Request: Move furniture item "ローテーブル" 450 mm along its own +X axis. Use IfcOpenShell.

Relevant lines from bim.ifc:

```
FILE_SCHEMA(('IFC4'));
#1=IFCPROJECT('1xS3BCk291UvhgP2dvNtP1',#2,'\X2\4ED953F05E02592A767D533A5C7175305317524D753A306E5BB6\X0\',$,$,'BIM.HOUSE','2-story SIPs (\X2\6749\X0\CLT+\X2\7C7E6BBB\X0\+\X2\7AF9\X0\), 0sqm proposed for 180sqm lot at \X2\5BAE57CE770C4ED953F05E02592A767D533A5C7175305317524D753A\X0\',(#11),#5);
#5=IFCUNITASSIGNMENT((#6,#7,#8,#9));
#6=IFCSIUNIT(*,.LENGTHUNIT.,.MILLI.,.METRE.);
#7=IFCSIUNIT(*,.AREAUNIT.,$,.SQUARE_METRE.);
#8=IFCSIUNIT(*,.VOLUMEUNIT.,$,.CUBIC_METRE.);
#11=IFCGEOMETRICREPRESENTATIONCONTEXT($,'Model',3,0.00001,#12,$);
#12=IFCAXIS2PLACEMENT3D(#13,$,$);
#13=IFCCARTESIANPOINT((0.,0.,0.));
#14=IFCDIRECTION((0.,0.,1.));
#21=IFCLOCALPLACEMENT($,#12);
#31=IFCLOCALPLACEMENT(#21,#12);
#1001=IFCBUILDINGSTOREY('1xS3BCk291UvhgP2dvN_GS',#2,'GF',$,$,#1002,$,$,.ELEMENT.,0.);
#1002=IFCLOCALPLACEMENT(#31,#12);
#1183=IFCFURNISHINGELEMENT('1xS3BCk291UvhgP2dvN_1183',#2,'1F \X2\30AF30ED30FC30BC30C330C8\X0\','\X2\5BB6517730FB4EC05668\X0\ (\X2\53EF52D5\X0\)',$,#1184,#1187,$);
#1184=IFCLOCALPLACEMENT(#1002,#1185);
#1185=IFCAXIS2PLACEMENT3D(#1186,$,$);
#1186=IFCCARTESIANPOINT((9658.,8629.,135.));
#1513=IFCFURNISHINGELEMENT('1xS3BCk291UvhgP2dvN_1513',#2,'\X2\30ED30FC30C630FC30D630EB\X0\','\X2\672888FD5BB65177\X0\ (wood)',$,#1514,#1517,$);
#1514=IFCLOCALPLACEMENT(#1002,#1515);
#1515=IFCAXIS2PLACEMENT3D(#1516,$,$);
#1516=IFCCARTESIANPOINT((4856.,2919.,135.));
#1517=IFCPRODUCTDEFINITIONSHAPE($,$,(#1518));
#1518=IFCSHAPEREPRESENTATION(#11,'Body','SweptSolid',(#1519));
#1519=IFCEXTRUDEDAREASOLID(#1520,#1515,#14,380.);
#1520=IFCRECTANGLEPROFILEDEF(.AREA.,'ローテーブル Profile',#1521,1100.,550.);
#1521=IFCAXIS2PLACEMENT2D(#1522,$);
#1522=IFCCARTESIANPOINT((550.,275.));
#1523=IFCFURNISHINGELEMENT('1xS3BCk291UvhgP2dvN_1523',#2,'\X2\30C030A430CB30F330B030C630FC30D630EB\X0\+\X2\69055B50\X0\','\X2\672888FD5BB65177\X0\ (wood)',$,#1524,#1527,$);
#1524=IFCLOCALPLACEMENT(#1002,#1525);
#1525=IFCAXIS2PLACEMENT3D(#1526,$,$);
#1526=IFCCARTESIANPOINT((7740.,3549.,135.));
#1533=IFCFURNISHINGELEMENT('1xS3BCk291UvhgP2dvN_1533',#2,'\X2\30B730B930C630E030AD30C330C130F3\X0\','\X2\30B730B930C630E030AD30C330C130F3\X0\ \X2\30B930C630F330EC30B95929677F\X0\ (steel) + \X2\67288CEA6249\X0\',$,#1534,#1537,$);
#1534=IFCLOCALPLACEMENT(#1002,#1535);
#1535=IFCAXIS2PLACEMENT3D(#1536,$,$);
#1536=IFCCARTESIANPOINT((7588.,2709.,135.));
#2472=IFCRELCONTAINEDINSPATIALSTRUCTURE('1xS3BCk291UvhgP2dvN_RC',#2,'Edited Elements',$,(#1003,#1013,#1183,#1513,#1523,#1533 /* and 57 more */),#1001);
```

```python
import ifcopenshell
import ifcopenshell.api.geometry
import ifcopenshell.util.placement
import ifcopenshell.util.unit

model = ifcopenshell.open("bim.ifc")
unit_scale = ifcopenshell.util.unit.calculate_unit_scale(model)

item = model.by_id(1513)
matrix = ifcopenshell.util.placement.get_local_placement(item.ObjectPlacement)
matrix[:3, 3] += matrix[:3, 0] * 0.45 / unit_scale
ifcopenshell.api.geometry.edit_object_placement(model, product=item, matrix=matrix, is_si=False)

print(ifcopenshell.util.placement.get_local_placement(item.ObjectPlacement).round(3) + 0.0)

model.write("bim_edited.ifc")
```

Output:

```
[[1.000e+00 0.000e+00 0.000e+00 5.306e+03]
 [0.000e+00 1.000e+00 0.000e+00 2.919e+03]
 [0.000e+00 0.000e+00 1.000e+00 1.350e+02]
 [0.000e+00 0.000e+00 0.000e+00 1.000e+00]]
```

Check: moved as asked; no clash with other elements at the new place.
